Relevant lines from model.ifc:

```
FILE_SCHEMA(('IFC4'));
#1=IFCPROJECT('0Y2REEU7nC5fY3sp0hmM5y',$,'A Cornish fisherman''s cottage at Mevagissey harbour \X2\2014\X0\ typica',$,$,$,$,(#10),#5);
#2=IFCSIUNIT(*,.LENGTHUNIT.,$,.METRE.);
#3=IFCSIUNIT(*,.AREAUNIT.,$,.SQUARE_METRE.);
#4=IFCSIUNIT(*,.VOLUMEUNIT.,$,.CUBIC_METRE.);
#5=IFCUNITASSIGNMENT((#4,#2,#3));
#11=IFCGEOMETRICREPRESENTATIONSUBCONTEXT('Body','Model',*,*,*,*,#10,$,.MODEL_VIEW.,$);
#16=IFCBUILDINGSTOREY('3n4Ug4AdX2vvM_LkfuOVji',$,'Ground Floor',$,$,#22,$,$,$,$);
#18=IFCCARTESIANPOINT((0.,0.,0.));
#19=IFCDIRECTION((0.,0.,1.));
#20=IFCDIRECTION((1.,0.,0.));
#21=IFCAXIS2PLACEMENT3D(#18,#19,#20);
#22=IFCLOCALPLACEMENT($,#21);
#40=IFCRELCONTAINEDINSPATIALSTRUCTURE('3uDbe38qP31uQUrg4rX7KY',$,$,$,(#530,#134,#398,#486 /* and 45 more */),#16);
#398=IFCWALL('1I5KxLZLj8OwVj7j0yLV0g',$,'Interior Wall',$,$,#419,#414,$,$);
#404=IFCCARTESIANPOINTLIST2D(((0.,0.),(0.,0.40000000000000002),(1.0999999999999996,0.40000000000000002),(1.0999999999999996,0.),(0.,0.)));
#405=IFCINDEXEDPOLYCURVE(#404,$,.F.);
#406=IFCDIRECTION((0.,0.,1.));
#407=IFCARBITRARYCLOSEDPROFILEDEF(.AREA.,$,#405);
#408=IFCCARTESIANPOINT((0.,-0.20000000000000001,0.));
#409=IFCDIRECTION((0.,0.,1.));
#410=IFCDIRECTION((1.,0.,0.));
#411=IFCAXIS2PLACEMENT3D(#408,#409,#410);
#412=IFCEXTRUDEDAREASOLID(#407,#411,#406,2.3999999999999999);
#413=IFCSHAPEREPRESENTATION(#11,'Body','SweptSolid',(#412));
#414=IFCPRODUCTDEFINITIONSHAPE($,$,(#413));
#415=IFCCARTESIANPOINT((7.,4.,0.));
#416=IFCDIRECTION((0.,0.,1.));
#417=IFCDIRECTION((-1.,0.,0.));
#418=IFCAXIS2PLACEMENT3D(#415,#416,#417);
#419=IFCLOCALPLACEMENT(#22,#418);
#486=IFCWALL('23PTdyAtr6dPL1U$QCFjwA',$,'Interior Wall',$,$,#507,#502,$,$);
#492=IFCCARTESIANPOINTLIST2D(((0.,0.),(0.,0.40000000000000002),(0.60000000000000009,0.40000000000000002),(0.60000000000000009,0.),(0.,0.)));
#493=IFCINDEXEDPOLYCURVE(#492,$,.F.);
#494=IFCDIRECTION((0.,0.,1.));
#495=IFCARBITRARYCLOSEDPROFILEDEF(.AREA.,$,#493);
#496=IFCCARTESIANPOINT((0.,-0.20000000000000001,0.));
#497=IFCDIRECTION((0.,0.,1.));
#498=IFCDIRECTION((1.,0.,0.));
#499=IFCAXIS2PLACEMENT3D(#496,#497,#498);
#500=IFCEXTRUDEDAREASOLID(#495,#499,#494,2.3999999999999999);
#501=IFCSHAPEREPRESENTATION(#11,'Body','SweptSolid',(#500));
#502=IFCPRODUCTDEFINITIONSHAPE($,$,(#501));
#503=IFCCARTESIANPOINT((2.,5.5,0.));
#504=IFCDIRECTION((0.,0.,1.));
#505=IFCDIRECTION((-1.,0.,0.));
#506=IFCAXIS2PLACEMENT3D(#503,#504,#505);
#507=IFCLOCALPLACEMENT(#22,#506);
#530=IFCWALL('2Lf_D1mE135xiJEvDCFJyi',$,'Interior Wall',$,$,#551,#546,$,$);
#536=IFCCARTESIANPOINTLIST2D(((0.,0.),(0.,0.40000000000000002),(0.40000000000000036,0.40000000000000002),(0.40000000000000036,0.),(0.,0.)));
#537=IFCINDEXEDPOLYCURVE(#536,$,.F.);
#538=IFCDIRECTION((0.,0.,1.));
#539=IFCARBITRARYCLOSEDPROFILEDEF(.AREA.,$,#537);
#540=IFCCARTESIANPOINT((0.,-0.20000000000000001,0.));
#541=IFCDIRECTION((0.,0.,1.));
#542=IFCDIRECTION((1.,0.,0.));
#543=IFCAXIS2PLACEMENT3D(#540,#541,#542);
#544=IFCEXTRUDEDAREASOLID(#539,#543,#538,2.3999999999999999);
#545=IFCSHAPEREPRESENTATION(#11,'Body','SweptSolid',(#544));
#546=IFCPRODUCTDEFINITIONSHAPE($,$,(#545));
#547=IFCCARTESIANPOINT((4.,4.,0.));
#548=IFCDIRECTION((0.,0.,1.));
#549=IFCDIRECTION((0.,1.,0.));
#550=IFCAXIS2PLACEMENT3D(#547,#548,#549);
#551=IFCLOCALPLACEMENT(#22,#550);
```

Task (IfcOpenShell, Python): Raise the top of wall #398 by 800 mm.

```python
import ifcopenshell
import ifcopenshell.geom
import ifcopenshell.util.representation
import ifcopenshell.util.shape
import ifcopenshell.util.unit

model = ifcopenshell.open("model.ifc")
unit_scale = ifcopenshell.util.unit.calculate_unit_scale(model)
settings = ifcopenshell.geom.settings()


def volume(element):
    """Net volume in cubic metres, openings subtracted."""
    shape = ifcopenshell.geom.create_shape(settings, element)
    return ifcopenshell.util.shape.get_volume(shape.geometry)


wall = model.by_guid("1I5KxLZLj8OwVj7j0yLV0g")
before = volume(wall)

body = ifcopenshell.util.representation.get_representation(wall, "Model", "Body")
solid = body.Items[0]
old_height = solid.Depth
solid.Depth += 0.8 / unit_scale
after = volume(wall)

print(f"height {old_height:g} -> {solid.Depth:g}, volume {before:.3f} -> {after:.3f} m3")

model.write("model-out.ifc")
```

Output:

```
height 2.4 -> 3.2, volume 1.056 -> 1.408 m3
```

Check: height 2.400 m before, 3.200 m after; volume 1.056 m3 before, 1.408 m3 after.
